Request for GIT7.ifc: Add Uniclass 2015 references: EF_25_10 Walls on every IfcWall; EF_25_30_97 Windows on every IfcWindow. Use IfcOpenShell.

First a look at what the model holds.

```python
import ifcopenshell

model = ifcopenshell.open("GIT7.ifc")
print(model.schema)
print("classifications:", [c.Name for c in model.by_type("IfcClassification")])
for ifc_class in ("IfcDoor", "IfcRoof", "IfcStair", "IfcWall", "IfcWindow"):
    print(ifc_class, len(model.by_type(ifc_class)))
```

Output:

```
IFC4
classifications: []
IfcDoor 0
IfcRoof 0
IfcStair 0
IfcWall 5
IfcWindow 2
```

```python
import ifcopenshell
import ifcopenshell.api.classification

model = ifcopenshell.open("GIT7.ifc")

system = ifcopenshell.api.classification.add_classification(model, classification="Uniclass 2015")

codes = {
    "IfcWall": ("EF_25_10", "Walls"),
    "IfcWindow": ("EF_25_30_97", "Windows"),
}
for ifc_class, (code, name) in codes.items():
    products = model.by_type(ifc_class)
    ifcopenshell.api.classification.add_reference(
        model, products=products, classification=system, identification=code, name=name
    )
    print(code, len(products))

model.write("GIT7_edited.ifc")
```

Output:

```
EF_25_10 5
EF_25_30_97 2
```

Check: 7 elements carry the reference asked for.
